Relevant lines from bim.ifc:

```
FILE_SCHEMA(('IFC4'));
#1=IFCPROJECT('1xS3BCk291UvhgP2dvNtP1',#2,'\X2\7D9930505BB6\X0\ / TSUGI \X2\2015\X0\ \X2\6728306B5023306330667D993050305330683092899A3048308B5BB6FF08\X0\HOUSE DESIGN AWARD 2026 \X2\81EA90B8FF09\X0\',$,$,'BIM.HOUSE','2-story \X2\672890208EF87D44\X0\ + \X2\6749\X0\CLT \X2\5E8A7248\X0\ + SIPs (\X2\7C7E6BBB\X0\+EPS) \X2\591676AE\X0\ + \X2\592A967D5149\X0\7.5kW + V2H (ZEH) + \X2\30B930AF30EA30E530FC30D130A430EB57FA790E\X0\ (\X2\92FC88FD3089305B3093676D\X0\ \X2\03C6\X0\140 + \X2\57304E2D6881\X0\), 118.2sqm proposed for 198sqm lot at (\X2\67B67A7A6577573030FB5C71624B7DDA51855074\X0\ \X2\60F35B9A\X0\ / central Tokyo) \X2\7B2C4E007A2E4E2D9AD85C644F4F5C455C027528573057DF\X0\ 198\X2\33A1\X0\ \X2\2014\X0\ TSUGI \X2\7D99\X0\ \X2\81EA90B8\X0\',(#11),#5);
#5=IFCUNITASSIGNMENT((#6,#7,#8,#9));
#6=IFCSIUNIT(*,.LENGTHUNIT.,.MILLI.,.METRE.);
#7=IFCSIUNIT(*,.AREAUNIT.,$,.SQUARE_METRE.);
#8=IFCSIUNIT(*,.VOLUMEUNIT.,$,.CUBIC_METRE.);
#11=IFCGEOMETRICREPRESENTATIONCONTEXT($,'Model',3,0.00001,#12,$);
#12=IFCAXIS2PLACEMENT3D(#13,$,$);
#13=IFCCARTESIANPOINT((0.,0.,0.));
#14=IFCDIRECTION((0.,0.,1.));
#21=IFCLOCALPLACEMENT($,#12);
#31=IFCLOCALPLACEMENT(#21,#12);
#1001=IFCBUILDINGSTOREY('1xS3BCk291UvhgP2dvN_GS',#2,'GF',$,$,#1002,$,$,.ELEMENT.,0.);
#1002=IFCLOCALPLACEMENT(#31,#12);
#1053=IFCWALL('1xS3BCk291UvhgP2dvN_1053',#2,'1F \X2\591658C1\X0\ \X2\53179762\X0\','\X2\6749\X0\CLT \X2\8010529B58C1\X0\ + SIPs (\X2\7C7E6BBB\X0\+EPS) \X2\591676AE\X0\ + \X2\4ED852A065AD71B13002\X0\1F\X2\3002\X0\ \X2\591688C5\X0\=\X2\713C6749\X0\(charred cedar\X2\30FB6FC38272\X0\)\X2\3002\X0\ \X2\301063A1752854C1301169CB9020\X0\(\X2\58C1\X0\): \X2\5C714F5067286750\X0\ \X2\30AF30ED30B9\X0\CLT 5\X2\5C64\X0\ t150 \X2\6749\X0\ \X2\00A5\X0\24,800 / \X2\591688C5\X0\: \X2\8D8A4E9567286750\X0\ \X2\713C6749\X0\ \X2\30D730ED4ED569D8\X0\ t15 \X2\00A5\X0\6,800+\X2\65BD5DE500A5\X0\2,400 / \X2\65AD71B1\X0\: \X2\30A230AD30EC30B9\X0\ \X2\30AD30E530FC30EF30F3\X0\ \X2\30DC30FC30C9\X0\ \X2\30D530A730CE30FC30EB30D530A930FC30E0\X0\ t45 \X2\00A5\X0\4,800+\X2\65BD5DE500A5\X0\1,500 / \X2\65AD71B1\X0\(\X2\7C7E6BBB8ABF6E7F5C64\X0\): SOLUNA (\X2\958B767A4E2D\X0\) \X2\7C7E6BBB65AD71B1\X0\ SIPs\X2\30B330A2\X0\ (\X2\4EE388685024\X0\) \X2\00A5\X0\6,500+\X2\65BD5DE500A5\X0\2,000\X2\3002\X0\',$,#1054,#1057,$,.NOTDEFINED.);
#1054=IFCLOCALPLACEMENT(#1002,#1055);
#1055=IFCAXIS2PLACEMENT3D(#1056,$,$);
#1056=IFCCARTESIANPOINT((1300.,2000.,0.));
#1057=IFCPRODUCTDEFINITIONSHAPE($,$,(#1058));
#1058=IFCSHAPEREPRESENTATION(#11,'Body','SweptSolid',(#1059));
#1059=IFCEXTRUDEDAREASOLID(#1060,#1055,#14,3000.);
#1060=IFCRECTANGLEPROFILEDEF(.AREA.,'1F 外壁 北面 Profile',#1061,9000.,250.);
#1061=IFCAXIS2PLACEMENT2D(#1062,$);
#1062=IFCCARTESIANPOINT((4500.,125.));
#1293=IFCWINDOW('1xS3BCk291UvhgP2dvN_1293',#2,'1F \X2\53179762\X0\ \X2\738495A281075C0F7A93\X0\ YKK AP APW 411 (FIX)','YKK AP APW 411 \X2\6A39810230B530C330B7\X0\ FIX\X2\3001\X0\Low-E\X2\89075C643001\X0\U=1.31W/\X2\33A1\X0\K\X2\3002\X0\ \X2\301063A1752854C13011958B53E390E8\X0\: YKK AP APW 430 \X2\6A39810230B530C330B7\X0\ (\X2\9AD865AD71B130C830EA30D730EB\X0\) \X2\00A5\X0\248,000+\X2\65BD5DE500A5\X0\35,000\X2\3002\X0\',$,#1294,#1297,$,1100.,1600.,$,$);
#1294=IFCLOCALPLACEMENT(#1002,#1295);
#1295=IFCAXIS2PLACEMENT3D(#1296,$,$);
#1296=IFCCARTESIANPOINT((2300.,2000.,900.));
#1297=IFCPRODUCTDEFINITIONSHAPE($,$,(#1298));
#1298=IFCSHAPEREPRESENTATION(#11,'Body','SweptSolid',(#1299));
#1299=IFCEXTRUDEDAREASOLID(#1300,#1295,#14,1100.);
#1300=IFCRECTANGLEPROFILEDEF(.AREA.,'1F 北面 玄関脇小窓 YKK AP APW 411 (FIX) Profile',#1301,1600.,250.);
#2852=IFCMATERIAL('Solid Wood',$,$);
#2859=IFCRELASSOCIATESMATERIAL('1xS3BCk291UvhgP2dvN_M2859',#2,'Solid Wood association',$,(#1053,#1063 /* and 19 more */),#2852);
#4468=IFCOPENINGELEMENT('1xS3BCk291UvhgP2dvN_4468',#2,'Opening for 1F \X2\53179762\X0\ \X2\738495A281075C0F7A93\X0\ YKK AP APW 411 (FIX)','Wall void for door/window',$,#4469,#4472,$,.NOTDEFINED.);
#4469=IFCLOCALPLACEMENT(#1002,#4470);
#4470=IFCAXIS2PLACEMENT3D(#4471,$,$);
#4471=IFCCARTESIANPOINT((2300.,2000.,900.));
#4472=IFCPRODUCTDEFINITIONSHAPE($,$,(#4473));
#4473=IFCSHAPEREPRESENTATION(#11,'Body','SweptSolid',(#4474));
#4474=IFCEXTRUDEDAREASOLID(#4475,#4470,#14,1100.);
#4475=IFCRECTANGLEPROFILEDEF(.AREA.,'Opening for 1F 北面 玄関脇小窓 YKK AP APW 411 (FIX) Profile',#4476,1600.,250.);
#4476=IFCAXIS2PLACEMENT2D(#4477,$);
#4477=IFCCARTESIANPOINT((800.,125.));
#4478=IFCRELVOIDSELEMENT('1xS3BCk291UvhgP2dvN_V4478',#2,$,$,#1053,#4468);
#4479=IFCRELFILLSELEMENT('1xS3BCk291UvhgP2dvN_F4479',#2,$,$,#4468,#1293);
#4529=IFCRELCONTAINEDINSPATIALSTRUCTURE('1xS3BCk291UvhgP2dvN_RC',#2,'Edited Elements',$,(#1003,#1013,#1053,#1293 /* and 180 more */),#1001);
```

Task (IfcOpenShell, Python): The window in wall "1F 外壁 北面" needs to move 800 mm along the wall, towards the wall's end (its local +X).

```python
import ifcopenshell
import ifcopenshell.api.geometry
import ifcopenshell.util.placement
import ifcopenshell.util.unit

model = ifcopenshell.open("bim.ifc")
unit_scale = ifcopenshell.util.unit.calculate_unit_scale(model)

window = model.by_guid("1xS3BCk291UvhgP2dvN_1293")
opening = window.FillsVoids[0].RelatingOpeningElement
wall = opening.VoidsElements[0].RelatingBuildingElement

wall_matrix = ifcopenshell.util.placement.get_local_placement(wall.ObjectPlacement)
shift = wall_matrix[:3, 0] * 0.8 / unit_scale
before = ifcopenshell.util.placement.get_local_placement(window.ObjectPlacement)[:3, 3].copy()

# The window is not placed relative to its opening, so move both.
for product in (opening, window):
    matrix = ifcopenshell.util.placement.get_local_placement(product.ObjectPlacement)
    matrix[:3, 3] += shift
    ifcopenshell.api.geometry.edit_object_placement(model, product=product, matrix=matrix, is_si=False)

after = ifcopenshell.util.placement.get_local_placement(window.ObjectPlacement)[:3, 3]
print("window moved by", (after - before).round(3) + 0.0)

model.write("bim_rev.ifc")
```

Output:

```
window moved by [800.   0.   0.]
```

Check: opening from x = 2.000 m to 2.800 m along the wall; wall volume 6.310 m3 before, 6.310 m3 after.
